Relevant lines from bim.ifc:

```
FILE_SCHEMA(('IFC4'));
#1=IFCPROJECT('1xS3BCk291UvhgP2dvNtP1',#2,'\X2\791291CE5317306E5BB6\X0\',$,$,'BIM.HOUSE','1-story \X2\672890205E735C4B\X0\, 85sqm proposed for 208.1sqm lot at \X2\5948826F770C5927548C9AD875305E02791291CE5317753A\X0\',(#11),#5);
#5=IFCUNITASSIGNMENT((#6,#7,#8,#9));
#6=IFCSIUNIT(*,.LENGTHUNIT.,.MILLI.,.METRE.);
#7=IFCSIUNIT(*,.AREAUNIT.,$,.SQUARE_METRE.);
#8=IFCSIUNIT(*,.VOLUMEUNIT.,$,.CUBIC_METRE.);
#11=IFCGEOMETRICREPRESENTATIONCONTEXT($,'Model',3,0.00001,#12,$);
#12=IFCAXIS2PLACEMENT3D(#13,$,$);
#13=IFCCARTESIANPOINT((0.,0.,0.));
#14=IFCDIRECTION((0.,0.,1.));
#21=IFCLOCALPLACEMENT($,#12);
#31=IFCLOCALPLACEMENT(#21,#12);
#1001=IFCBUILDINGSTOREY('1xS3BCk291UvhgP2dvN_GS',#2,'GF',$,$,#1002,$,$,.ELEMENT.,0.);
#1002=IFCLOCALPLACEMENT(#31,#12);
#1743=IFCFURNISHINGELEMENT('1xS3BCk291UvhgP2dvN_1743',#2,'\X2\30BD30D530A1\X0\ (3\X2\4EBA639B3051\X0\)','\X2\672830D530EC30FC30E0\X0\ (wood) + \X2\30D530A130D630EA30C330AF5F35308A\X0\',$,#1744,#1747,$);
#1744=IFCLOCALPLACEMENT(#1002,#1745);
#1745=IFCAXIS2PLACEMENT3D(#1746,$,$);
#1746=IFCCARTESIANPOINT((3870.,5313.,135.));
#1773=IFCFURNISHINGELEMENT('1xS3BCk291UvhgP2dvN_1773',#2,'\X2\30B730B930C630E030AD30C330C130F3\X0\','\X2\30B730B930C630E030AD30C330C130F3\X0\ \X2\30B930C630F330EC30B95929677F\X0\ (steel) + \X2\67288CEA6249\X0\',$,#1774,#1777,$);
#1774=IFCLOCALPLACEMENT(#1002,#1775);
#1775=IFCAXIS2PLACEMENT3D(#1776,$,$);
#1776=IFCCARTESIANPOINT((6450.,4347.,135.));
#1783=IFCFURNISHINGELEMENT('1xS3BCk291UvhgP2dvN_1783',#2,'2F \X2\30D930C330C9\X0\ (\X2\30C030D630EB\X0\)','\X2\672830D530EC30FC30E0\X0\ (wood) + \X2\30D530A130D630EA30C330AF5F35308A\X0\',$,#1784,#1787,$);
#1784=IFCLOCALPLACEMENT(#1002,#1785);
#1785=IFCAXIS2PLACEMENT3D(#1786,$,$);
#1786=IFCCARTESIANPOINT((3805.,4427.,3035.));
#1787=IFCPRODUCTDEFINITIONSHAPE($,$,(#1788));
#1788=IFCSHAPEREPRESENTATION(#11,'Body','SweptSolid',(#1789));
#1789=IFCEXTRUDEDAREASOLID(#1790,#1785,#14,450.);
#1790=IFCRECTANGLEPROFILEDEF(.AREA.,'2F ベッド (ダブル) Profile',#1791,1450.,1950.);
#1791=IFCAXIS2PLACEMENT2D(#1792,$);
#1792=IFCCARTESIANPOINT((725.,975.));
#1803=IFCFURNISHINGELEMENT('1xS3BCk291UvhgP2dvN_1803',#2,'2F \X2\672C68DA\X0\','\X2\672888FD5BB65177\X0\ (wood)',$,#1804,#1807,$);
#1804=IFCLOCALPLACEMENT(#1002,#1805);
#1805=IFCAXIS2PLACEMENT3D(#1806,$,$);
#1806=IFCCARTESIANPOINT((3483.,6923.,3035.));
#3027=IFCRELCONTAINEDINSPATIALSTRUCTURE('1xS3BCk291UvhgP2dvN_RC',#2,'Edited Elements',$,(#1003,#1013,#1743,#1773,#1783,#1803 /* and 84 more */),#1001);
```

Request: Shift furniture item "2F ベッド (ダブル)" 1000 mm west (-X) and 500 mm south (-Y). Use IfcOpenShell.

```python
import ifcopenshell
import ifcopenshell.api.geometry
import ifcopenshell.util.placement

model = ifcopenshell.open("bim.ifc")

item = model.by_guid("1xS3BCk291UvhgP2dvN_1783")
matrix = ifcopenshell.util.placement.get_local_placement(item.ObjectPlacement)
matrix[0, 3] -= 1000.0
matrix[1, 3] -= 500.0
ifcopenshell.api.geometry.edit_object_placement(model, product=item, matrix=matrix, is_si=False)

print(ifcopenshell.util.placement.get_local_placement(item.ObjectPlacement).round(3) + 0.0)

model.write("bim-out.ifc")
```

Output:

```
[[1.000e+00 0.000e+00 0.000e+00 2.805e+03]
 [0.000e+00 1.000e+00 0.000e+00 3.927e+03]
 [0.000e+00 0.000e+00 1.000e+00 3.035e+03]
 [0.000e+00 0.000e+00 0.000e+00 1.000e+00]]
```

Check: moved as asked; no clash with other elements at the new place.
